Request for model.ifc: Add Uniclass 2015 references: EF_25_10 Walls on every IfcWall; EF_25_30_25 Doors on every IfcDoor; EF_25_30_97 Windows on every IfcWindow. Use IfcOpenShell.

First a look at what the model holds.

```python
import ifcopenshell

model = ifcopenshell.open("model.ifc")
print(model.schema)
print("classifications:", [c.Name for c in model.by_type("IfcClassification")])
for ifc_class in ("IfcDoor", "IfcRoof", "IfcStair", "IfcWall", "IfcWindow"):
    print(ifc_class, len(model.by_type(ifc_class)))
```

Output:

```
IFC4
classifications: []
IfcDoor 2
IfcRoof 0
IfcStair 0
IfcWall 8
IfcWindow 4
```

```python
import ifcopenshell
import ifcopenshell.api.classification

model = ifcopenshell.open("model.ifc")

system = ifcopenshell.api.classification.add_classification(model, classification="Uniclass 2015")

codes = {
    "IfcWall": ("EF_25_10", "Walls"),
    "IfcDoor": ("EF_25_30_25", "Doors"),
    "IfcWindow": ("EF_25_30_97", "Windows"),
}
for ifc_class, (code, name) in codes.items():
    products = model.by_type(ifc_class)
    ifcopenshell.api.classification.add_reference(
        model, products=products, classification=system, identification=code, name=name
    )
    print(code, len(products))

model.write("model_edited.ifc")
```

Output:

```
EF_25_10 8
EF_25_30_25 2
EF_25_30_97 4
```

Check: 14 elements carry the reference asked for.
